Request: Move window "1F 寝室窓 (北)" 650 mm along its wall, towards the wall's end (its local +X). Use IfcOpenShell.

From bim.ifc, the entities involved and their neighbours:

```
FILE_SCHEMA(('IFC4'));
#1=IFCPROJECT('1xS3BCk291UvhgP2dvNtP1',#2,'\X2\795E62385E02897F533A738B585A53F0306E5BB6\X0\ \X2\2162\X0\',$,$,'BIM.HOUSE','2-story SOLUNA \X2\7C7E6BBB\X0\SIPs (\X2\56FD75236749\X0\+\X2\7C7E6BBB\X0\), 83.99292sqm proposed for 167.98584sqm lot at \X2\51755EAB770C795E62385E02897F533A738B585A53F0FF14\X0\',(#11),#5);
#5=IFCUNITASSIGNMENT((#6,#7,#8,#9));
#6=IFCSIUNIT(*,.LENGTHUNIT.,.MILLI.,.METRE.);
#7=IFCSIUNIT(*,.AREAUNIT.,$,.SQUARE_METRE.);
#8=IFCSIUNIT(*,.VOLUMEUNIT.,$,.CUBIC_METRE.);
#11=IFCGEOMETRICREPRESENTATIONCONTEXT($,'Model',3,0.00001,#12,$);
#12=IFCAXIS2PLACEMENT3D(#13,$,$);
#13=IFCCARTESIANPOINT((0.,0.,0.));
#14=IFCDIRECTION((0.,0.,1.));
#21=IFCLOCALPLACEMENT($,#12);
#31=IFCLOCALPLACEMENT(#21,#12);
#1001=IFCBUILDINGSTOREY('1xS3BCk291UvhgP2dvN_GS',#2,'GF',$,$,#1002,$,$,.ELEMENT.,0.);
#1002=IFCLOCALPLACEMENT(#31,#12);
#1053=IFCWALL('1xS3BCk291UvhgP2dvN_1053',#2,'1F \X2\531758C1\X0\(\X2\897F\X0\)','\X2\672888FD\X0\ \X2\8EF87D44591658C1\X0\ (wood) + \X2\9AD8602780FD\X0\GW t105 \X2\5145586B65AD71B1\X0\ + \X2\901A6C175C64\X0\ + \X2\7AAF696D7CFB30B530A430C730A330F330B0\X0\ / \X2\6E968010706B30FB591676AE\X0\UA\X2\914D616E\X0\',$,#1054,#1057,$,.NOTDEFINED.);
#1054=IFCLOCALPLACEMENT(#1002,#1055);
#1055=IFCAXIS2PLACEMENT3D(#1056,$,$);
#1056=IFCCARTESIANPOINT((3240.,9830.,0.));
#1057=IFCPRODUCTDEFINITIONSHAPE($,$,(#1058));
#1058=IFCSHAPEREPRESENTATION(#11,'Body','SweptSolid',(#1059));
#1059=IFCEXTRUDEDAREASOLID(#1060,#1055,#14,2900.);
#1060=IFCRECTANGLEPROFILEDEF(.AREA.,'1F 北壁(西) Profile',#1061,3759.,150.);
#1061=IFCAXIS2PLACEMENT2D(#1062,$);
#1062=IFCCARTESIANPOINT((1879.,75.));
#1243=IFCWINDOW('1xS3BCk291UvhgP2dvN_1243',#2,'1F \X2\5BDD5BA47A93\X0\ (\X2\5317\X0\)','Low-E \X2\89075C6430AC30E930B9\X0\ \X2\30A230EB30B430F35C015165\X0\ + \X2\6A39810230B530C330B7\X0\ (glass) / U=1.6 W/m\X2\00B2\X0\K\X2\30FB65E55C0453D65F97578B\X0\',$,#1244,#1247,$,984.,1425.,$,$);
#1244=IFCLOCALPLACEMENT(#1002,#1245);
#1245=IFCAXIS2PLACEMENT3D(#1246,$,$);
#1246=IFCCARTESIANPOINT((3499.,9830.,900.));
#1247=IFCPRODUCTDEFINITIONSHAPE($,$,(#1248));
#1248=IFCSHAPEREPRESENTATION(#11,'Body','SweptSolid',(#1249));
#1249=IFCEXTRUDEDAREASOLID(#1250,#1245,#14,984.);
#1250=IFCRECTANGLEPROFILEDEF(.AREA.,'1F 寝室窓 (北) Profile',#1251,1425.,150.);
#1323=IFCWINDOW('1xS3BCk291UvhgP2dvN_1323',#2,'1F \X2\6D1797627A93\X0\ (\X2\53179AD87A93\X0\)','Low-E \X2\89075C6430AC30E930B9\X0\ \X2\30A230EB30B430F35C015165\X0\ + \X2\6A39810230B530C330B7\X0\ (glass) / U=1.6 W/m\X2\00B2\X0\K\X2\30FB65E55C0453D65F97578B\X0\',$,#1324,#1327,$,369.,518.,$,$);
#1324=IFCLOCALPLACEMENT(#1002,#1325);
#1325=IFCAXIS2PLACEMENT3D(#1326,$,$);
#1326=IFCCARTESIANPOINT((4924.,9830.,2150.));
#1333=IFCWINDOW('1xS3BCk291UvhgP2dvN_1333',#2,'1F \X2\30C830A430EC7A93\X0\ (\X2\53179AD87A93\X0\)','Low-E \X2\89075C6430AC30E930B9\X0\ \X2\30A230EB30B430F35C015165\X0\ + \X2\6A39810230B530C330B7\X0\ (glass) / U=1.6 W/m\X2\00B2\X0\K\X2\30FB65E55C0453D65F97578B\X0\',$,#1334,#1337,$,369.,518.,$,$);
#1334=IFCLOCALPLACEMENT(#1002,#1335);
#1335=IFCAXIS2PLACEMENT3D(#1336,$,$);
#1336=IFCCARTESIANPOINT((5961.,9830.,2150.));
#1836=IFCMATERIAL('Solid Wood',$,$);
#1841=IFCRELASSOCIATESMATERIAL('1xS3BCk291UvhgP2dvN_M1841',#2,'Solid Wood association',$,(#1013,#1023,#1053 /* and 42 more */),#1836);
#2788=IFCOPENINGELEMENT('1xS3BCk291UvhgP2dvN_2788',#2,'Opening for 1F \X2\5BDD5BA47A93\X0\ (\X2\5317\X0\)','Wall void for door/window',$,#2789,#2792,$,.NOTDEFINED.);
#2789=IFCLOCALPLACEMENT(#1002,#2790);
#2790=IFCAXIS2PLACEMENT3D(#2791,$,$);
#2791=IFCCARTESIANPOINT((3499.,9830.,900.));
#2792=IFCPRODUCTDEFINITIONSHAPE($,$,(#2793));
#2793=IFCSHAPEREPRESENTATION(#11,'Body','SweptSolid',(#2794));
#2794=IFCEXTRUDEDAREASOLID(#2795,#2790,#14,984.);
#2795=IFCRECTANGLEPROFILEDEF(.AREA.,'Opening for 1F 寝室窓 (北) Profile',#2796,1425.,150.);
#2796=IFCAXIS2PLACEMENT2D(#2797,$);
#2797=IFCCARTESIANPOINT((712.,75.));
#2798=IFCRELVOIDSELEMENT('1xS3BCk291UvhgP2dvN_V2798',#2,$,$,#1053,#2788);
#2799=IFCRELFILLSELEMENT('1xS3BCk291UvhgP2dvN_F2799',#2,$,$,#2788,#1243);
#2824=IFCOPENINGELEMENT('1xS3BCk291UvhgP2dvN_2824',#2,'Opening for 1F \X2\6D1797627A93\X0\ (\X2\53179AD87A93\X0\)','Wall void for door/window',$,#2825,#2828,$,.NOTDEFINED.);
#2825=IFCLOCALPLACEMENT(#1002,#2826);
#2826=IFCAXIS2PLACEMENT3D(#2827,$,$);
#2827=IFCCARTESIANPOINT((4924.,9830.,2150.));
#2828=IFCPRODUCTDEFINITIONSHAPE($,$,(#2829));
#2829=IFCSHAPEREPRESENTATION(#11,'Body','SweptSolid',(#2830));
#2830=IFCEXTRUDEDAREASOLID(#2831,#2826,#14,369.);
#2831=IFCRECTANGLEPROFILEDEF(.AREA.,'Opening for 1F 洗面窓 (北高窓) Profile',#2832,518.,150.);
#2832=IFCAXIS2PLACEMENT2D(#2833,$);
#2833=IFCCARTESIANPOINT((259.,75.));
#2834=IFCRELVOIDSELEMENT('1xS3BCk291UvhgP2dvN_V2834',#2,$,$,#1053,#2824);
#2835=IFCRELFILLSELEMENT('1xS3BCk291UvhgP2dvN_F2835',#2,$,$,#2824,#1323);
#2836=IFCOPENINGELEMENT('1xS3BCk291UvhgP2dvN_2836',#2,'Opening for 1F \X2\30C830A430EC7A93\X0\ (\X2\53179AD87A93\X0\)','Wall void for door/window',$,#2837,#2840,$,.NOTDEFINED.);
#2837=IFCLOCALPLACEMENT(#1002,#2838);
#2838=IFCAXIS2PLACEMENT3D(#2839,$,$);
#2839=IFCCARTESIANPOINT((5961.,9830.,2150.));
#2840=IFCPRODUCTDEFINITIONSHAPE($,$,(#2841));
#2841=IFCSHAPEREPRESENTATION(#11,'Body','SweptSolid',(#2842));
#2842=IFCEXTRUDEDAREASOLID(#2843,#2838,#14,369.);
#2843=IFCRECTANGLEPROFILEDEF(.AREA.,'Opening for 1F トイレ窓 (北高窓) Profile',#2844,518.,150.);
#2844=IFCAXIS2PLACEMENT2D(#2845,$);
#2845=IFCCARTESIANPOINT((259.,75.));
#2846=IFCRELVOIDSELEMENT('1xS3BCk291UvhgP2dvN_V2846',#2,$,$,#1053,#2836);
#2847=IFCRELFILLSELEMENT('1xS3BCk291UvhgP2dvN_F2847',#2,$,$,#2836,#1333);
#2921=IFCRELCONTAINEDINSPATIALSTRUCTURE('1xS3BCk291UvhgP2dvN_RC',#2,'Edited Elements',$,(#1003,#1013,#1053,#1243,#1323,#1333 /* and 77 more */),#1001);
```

```python
import ifcopenshell
import ifcopenshell.api.geometry
import ifcopenshell.util.placement

model = ifcopenshell.open("bim.ifc")

window = model.by_id(1243)
opening = window.FillsVoids[0].RelatingOpeningElement
wall = opening.VoidsElements[0].RelatingBuildingElement

wall_matrix = ifcopenshell.util.placement.get_local_placement(wall.ObjectPlacement)
shift = wall_matrix[:3, 0] * 650.0
before = ifcopenshell.util.placement.get_local_placement(window.ObjectPlacement)[:3, 3].copy()

# The window is not placed relative to its opening, so move both.
for product in (opening, window):
    matrix = ifcopenshell.util.placement.get_local_placement(product.ObjectPlacement)
    matrix[:3, 3] += shift
    ifcopenshell.api.geometry.edit_object_placement(model, product=product, matrix=matrix, is_si=False)

after = ifcopenshell.util.placement.get_local_placement(window.ObjectPlacement)[:3, 3]
print("window moved by", (after - before).round(3) + 0.0)

model.write("bim-out.ifc")
```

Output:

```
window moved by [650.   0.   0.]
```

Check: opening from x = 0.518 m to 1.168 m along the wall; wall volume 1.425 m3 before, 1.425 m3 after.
